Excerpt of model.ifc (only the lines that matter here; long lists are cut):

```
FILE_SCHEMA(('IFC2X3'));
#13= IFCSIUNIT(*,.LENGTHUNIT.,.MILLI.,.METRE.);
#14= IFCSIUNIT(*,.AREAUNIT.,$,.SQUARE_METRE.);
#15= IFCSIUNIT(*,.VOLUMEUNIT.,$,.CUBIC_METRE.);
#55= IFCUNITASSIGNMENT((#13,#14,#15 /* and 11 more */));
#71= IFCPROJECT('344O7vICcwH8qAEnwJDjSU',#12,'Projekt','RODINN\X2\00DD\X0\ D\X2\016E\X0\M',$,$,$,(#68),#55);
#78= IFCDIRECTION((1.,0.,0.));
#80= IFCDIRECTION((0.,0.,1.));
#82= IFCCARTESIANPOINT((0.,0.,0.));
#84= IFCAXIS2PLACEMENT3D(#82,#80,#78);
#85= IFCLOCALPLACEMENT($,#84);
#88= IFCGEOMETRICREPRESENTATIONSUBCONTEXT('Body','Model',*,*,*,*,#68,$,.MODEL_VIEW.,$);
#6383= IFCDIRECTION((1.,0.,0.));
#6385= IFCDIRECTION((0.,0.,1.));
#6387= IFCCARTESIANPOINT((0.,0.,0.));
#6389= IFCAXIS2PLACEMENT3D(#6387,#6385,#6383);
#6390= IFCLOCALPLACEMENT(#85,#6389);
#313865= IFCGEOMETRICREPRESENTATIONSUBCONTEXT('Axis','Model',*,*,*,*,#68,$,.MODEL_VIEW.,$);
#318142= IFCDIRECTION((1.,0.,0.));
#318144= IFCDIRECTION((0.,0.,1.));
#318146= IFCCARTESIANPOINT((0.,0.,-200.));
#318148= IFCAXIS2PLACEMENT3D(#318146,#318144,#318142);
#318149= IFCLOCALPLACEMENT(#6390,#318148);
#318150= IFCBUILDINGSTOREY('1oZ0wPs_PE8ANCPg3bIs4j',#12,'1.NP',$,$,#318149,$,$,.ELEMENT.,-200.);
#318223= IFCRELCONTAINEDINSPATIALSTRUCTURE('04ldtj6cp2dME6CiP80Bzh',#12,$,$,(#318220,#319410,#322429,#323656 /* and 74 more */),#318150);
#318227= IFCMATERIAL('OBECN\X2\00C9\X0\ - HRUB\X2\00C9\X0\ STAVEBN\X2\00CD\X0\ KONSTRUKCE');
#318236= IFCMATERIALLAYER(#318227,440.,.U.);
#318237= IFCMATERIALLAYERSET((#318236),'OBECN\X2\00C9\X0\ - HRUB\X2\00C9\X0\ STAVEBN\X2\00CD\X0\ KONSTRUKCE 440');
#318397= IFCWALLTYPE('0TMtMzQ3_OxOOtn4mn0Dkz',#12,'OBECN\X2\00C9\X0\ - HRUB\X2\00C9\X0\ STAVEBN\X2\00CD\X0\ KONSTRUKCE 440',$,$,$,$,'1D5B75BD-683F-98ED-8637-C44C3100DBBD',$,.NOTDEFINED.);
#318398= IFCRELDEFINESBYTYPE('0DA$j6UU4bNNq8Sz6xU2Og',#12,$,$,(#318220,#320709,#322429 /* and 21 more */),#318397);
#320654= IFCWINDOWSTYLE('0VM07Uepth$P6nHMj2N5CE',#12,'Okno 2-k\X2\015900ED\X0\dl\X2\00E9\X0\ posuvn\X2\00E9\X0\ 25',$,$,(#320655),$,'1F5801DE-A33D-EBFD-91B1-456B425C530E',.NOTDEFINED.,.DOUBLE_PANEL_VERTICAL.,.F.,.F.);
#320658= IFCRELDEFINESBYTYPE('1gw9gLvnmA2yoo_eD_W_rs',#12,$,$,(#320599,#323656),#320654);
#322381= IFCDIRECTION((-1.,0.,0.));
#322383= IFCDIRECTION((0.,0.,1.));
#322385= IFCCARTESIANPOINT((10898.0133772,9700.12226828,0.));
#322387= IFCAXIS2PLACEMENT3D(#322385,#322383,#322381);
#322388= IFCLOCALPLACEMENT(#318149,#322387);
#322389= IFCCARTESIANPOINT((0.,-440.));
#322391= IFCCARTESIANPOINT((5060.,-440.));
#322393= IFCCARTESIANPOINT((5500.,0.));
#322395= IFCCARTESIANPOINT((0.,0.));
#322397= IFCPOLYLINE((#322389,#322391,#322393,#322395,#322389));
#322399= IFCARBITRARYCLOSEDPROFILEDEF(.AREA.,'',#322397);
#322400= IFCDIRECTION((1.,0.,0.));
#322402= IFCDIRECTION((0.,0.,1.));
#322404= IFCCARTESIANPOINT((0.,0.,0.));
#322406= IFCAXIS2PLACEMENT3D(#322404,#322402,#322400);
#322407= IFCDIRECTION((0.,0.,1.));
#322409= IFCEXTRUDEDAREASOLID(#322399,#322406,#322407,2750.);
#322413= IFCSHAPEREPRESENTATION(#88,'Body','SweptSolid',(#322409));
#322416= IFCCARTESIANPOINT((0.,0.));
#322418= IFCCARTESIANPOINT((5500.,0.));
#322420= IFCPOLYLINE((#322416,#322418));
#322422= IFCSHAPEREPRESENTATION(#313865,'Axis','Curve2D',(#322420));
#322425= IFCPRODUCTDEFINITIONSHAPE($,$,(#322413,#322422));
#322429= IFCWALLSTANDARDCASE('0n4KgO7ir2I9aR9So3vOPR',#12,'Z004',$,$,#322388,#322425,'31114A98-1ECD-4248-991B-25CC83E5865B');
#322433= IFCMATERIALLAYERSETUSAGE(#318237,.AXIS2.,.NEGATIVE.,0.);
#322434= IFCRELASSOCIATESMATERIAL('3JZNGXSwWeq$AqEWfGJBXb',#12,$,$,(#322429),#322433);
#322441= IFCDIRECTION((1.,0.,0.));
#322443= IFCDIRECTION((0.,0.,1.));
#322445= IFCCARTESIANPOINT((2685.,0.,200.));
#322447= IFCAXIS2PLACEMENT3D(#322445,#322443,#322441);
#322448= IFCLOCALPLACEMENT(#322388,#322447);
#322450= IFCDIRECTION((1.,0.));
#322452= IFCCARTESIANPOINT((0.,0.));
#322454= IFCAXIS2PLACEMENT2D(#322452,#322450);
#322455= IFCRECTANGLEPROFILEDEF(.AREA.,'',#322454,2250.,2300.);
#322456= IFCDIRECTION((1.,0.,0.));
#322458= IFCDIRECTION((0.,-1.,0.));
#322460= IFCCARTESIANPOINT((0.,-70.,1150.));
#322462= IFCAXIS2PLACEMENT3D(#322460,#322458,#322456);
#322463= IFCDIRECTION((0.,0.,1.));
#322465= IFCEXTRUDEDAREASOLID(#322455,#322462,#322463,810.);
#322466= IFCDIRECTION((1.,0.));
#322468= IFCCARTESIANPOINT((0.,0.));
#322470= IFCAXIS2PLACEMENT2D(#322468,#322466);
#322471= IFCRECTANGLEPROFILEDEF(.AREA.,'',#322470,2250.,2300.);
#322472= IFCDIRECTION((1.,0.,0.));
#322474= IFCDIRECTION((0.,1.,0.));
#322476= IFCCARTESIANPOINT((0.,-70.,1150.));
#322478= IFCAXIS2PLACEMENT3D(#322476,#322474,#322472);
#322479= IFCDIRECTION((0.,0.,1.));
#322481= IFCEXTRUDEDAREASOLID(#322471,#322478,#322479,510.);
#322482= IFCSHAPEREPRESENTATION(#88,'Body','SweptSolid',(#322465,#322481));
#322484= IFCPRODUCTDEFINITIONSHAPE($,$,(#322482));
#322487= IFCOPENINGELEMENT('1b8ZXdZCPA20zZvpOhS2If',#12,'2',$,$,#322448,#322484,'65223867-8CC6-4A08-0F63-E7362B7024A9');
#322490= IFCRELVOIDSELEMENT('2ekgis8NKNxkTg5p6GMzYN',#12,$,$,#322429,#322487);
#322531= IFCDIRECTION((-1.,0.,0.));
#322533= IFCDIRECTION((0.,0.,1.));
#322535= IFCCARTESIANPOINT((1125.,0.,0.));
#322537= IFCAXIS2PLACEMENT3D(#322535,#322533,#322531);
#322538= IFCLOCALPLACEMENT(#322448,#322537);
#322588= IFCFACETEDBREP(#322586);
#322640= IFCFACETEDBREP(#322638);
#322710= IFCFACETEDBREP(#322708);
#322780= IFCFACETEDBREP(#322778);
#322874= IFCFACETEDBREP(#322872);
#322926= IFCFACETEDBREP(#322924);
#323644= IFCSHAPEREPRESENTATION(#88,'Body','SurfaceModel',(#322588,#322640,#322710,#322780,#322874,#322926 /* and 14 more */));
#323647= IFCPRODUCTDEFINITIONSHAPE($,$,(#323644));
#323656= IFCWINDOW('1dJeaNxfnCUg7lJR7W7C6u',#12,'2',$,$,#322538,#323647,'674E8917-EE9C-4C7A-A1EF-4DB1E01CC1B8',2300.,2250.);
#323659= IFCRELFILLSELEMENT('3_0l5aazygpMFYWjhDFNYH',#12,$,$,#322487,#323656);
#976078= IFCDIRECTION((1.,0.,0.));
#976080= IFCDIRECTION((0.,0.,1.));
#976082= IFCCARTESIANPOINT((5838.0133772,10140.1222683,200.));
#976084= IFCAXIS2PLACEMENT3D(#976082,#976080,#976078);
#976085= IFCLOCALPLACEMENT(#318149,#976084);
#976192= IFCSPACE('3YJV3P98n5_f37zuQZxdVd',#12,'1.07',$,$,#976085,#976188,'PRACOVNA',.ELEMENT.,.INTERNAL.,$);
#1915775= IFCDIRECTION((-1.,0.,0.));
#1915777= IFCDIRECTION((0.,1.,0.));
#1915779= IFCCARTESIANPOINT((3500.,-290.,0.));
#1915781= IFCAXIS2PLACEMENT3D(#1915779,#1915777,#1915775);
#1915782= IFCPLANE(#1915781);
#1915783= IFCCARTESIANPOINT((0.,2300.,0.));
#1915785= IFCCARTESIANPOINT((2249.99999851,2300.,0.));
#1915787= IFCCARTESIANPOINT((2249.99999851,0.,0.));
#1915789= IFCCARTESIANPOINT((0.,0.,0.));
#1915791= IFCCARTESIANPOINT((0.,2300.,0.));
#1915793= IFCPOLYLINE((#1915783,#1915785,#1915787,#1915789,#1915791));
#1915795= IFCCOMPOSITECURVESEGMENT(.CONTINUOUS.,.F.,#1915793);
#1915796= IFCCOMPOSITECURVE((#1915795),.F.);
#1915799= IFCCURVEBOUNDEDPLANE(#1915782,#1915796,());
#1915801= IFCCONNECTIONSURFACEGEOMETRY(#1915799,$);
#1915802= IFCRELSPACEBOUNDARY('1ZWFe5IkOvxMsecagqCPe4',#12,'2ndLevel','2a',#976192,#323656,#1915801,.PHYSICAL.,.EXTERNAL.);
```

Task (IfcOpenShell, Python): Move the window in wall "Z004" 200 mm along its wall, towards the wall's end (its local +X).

```python
import numpy as np
import ifcopenshell
import ifcopenshell.api.geometry
import ifcopenshell.util.placement
import ifcopenshell.util.unit

model = ifcopenshell.open("model.ifc")
unit_scale = ifcopenshell.util.unit.calculate_unit_scale(model)

window = model.by_guid("1dJeaNxfnCUg7lJR7W7C6u")
opening = window.FillsVoids[0].RelatingOpeningElement
wall = opening.VoidsElements[0].RelatingBuildingElement

wall_matrix = ifcopenshell.util.placement.get_local_placement(wall.ObjectPlacement)
shift = wall_matrix[:3, 0] * 0.2 / unit_scale
before = ifcopenshell.util.placement.get_local_placement(window.ObjectPlacement)[:3, 3].copy()

# The window is placed relative to its opening, so it follows when the opening moves.
matrix = ifcopenshell.util.placement.get_local_placement(opening.ObjectPlacement)
matrix[:3, 3] += shift
ifcopenshell.api.geometry.edit_object_placement(
    model, product=opening, matrix=matrix, is_si=False, should_transform_children=True
)

# Space boundary surfaces are stored in each space's coordinates; move them too.
for rel in window.ProvidesBoundaries:
    if not rel.ConnectionGeometry:
        continue
    surface = rel.ConnectionGeometry.SurfaceOnRelatingElement.BasisSurface
    space_matrix = ifcopenshell.util.placement.get_local_placement(rel.RelatingSpace.ObjectPlacement)
    point = np.array(surface.Position.Location.Coordinates) + space_matrix[:3, :3].T @ shift
    surface.Position = model.createIfcAxis2Placement3D(
        model.createIfcCartesianPoint(point.tolist()), surface.Position.Axis, surface.Position.RefDirection
    )

after = ifcopenshell.util.placement.get_local_placement(window.ObjectPlacement)[:3, 3]
print("window moved by", (after - before).round(3) + 0.0)

model.write("model_v2.ifc")
```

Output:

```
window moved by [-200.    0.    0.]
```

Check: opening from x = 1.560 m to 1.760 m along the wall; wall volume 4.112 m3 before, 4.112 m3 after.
